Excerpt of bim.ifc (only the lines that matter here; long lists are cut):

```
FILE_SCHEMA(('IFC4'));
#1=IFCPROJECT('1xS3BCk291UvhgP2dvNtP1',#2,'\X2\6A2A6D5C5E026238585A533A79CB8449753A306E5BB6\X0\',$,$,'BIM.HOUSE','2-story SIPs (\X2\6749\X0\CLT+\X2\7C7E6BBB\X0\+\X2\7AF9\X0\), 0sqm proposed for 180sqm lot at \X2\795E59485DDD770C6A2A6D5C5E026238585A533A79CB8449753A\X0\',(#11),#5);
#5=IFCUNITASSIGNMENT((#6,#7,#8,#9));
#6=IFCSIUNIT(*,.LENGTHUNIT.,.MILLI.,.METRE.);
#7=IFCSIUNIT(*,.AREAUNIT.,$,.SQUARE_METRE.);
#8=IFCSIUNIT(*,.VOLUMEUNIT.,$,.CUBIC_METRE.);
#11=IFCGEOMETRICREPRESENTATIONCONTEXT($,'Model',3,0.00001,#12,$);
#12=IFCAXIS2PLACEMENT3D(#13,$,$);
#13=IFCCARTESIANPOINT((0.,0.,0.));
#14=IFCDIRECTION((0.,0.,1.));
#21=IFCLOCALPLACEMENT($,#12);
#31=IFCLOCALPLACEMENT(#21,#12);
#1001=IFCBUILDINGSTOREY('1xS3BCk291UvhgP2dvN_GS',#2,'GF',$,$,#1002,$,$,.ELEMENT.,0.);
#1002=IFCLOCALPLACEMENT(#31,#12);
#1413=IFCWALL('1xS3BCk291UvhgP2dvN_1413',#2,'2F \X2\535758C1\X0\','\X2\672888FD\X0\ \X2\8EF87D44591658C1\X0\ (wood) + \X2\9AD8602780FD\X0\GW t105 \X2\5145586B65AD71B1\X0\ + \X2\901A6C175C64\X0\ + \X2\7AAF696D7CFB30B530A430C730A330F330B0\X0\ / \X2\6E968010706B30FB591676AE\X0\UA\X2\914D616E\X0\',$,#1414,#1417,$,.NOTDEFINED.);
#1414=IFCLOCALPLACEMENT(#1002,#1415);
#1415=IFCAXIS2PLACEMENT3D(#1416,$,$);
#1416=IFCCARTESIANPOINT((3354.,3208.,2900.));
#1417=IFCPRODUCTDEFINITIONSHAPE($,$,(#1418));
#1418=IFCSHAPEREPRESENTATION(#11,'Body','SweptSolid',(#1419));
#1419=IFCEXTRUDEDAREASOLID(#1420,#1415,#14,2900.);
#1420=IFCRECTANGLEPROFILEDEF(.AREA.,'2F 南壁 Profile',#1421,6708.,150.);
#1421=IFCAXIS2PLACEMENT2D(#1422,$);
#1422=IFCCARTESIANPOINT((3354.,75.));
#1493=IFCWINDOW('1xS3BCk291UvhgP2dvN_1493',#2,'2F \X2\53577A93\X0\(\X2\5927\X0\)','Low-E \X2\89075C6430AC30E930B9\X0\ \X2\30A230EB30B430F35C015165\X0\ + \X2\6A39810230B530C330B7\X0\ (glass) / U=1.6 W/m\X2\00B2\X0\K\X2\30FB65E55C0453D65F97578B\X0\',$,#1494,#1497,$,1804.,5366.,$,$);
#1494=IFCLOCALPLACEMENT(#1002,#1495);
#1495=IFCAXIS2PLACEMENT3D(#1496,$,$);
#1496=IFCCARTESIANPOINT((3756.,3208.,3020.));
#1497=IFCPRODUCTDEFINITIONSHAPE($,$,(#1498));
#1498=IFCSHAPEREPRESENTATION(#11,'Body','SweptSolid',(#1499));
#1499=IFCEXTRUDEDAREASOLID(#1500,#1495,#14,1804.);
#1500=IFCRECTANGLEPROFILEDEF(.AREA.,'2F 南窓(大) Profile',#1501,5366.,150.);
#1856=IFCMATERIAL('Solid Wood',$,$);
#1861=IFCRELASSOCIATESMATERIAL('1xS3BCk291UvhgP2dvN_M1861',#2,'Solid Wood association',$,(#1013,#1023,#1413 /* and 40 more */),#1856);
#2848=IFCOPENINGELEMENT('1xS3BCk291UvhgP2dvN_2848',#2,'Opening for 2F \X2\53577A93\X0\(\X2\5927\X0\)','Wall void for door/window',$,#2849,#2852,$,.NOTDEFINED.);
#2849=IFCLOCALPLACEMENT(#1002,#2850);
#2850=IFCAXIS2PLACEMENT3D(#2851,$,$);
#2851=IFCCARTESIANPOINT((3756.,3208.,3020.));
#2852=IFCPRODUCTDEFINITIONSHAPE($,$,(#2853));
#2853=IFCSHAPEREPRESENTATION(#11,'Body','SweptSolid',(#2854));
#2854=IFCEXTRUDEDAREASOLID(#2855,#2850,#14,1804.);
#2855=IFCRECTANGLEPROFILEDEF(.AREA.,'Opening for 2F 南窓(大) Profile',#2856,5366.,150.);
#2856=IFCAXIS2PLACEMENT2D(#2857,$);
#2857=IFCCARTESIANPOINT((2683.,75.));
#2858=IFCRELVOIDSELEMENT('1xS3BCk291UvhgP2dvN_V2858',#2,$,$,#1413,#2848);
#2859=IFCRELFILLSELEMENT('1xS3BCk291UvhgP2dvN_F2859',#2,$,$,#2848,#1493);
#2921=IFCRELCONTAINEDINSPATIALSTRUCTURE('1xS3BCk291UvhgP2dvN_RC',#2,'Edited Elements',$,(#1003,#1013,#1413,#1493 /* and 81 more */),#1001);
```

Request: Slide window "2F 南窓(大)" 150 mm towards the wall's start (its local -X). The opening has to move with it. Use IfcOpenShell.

```python
import ifcopenshell
import ifcopenshell.api.geometry
import ifcopenshell.util.placement
import ifcopenshell.util.unit

model = ifcopenshell.open("bim.ifc")
unit_scale = ifcopenshell.util.unit.calculate_unit_scale(model)

window = model.by_guid("1xS3BCk291UvhgP2dvN_1493")
opening = window.FillsVoids[0].RelatingOpeningElement
wall = opening.VoidsElements[0].RelatingBuildingElement

wall_matrix = ifcopenshell.util.placement.get_local_placement(wall.ObjectPlacement)
shift = wall_matrix[:3, 0] * -0.15 / unit_scale
before = ifcopenshell.util.placement.get_local_placement(window.ObjectPlacement)[:3, 3].copy()

# The window is not placed relative to its opening, so move both.
for product in (opening, window):
    matrix = ifcopenshell.util.placement.get_local_placement(product.ObjectPlacement)
    matrix[:3, 3] += shift
    ifcopenshell.api.geometry.edit_object_placement(model, product=product, matrix=matrix, is_si=False)

after = ifcopenshell.util.placement.get_local_placement(window.ObjectPlacement)[:3, 3]
print("window moved by", (after - before).round(3) + 0.0)

model.write("bim_updated.ifc")
```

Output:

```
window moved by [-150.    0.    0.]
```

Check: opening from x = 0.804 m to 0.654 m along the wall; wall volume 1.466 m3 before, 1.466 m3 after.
